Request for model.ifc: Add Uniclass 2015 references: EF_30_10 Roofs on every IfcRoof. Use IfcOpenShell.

First a look at what the model holds.

```python
import ifcopenshell

model = ifcopenshell.open("model.ifc")
print(model.schema)
print("classifications:", [c.Name for c in model.by_type("IfcClassification")])
for ifc_class in ("IfcDoor", "IfcRoof", "IfcStair", "IfcWall", "IfcWindow"):
    print(ifc_class, len(model.by_type(ifc_class)))
```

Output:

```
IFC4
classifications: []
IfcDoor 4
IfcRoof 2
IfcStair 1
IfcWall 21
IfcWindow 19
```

```python
import ifcopenshell
import ifcopenshell.api.classification

model = ifcopenshell.open("model.ifc")

system = ifcopenshell.api.classification.add_classification(model, classification="Uniclass 2015")

codes = {
    "IfcRoof": ("EF_30_10", "Roofs"),
}
for ifc_class, (code, name) in codes.items():
    products = model.by_type(ifc_class)
    ifcopenshell.api.classification.add_reference(
        model, products=products, classification=system, identification=code, name=name
    )
    print(code, len(products))

model.write("model_rev.ifc")
```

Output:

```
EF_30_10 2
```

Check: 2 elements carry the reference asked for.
